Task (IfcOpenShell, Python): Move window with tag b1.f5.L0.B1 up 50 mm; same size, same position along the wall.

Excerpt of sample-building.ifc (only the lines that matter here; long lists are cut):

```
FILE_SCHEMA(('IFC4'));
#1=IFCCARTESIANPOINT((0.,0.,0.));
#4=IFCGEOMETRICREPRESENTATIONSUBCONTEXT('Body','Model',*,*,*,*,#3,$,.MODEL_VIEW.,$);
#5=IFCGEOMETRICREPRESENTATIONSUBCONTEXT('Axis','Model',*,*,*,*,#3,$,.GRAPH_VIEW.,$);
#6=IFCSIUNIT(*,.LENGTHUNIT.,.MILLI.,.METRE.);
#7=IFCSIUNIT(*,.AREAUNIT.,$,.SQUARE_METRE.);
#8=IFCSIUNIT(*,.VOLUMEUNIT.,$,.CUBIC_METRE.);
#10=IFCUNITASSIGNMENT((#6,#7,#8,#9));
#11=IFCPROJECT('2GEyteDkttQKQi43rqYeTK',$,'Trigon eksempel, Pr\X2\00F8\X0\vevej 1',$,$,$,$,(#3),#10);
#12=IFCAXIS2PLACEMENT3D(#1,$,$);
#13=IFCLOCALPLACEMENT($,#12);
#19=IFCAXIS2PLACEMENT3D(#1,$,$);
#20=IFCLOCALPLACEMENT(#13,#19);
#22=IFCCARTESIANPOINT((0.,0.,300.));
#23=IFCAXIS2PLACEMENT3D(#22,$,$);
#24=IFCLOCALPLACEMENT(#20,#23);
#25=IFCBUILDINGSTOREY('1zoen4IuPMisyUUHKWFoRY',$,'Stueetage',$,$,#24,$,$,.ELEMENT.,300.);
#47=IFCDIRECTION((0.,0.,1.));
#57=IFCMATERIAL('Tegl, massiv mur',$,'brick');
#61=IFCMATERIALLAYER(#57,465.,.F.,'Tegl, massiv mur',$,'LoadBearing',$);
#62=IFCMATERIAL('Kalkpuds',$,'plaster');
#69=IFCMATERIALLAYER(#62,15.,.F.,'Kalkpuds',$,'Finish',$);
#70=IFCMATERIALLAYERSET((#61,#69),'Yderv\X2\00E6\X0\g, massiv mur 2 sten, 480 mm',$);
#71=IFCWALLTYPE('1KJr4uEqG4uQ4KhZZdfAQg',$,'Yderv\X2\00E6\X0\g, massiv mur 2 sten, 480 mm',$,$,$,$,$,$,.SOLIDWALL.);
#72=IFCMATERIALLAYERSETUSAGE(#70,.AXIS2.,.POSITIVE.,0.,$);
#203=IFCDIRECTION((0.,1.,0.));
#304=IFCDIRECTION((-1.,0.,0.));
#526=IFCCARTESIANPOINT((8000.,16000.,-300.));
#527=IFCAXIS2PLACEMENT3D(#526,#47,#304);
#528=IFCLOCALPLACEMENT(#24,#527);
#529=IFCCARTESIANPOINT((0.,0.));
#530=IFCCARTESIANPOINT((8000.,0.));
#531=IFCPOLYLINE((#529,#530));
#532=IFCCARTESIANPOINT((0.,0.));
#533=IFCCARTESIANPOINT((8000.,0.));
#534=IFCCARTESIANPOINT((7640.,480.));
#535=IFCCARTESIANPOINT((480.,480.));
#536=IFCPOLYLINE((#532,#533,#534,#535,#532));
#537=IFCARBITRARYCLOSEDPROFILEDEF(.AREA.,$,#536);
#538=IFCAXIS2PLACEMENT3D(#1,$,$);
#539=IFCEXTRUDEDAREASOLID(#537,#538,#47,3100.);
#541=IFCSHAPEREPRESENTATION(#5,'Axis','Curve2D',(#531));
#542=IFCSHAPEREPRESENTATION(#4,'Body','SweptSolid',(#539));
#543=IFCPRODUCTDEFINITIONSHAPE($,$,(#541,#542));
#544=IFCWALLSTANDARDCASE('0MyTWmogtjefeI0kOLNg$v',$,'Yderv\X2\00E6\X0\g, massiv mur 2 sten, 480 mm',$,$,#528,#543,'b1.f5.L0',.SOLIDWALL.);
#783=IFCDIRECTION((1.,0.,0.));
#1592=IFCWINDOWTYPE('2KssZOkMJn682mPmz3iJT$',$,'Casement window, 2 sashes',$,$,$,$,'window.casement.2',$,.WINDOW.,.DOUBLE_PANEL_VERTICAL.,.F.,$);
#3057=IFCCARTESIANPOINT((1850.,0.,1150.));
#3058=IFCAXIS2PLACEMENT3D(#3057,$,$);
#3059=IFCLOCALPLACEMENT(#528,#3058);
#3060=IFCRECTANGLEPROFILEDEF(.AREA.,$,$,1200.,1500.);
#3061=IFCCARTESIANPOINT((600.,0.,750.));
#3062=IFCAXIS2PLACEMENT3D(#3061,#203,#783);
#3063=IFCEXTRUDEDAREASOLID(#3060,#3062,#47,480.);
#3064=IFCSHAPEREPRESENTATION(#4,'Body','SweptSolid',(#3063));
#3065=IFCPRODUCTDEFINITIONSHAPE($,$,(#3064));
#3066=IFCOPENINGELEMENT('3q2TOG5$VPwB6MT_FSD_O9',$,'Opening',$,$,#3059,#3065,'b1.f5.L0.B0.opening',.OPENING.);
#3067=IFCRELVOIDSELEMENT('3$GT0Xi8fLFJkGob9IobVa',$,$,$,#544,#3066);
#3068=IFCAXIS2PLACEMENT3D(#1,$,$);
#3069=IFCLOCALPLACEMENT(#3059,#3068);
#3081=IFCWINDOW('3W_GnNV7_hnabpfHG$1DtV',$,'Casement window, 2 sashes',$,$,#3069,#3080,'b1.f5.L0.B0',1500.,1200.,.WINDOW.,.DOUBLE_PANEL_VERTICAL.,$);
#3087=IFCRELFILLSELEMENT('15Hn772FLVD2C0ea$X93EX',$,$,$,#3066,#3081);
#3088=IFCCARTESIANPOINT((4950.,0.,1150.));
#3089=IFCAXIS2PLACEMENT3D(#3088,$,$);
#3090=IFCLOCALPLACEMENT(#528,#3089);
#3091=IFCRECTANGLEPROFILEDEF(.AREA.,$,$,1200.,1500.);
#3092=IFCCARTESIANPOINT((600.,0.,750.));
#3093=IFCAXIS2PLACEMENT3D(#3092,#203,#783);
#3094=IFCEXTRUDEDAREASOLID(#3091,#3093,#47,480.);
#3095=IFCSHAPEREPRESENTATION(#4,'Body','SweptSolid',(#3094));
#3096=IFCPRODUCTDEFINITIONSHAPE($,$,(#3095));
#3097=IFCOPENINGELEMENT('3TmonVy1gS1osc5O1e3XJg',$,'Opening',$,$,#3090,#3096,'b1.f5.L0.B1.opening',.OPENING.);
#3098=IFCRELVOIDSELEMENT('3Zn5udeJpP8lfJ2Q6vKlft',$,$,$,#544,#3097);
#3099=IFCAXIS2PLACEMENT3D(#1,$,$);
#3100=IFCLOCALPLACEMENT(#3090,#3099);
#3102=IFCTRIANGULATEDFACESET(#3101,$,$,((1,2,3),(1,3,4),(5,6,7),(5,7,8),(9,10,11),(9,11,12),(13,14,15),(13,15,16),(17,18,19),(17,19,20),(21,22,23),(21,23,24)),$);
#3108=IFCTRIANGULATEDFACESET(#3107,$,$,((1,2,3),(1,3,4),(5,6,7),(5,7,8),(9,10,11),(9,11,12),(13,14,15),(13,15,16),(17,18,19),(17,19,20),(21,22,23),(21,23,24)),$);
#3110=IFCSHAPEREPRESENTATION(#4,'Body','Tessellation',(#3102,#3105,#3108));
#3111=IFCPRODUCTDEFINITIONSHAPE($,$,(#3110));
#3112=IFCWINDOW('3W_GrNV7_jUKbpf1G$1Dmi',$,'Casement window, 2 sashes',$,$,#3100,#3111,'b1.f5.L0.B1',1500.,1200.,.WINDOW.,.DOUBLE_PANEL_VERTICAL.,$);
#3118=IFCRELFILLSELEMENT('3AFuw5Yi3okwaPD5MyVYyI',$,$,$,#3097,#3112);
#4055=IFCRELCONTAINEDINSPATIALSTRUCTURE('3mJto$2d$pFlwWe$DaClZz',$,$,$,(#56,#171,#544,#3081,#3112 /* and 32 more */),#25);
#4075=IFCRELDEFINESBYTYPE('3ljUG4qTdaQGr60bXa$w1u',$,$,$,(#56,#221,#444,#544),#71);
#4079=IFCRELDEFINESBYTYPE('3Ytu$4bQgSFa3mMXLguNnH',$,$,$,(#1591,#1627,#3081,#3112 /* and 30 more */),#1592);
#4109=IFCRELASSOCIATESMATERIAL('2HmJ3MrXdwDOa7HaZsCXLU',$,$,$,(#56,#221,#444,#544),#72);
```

```python
import numpy as np
import ifcopenshell
import ifcopenshell.api.geometry
import ifcopenshell.util.placement
import ifcopenshell.util.unit

model = ifcopenshell.open("sample-building.ifc")
unit_scale = ifcopenshell.util.unit.calculate_unit_scale(model)

window = model.by_id(3112)
opening = window.FillsVoids[0].RelatingOpeningElement
dz = 0.05 / unit_scale

shift = np.array([0.0, 0.0, dz])
# The window is placed relative to its opening, so it follows when the opening moves.
matrix = ifcopenshell.util.placement.get_local_placement(opening.ObjectPlacement)
matrix[:3, 3] += shift
ifcopenshell.api.geometry.edit_object_placement(
    model, product=opening, matrix=matrix, is_si=False, should_transform_children=True
)

print(f"moved by {dz * unit_scale:+.3f} m")

model.write("sample-building_v2.ifc")
```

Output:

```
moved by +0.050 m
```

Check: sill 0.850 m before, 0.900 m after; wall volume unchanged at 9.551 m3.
